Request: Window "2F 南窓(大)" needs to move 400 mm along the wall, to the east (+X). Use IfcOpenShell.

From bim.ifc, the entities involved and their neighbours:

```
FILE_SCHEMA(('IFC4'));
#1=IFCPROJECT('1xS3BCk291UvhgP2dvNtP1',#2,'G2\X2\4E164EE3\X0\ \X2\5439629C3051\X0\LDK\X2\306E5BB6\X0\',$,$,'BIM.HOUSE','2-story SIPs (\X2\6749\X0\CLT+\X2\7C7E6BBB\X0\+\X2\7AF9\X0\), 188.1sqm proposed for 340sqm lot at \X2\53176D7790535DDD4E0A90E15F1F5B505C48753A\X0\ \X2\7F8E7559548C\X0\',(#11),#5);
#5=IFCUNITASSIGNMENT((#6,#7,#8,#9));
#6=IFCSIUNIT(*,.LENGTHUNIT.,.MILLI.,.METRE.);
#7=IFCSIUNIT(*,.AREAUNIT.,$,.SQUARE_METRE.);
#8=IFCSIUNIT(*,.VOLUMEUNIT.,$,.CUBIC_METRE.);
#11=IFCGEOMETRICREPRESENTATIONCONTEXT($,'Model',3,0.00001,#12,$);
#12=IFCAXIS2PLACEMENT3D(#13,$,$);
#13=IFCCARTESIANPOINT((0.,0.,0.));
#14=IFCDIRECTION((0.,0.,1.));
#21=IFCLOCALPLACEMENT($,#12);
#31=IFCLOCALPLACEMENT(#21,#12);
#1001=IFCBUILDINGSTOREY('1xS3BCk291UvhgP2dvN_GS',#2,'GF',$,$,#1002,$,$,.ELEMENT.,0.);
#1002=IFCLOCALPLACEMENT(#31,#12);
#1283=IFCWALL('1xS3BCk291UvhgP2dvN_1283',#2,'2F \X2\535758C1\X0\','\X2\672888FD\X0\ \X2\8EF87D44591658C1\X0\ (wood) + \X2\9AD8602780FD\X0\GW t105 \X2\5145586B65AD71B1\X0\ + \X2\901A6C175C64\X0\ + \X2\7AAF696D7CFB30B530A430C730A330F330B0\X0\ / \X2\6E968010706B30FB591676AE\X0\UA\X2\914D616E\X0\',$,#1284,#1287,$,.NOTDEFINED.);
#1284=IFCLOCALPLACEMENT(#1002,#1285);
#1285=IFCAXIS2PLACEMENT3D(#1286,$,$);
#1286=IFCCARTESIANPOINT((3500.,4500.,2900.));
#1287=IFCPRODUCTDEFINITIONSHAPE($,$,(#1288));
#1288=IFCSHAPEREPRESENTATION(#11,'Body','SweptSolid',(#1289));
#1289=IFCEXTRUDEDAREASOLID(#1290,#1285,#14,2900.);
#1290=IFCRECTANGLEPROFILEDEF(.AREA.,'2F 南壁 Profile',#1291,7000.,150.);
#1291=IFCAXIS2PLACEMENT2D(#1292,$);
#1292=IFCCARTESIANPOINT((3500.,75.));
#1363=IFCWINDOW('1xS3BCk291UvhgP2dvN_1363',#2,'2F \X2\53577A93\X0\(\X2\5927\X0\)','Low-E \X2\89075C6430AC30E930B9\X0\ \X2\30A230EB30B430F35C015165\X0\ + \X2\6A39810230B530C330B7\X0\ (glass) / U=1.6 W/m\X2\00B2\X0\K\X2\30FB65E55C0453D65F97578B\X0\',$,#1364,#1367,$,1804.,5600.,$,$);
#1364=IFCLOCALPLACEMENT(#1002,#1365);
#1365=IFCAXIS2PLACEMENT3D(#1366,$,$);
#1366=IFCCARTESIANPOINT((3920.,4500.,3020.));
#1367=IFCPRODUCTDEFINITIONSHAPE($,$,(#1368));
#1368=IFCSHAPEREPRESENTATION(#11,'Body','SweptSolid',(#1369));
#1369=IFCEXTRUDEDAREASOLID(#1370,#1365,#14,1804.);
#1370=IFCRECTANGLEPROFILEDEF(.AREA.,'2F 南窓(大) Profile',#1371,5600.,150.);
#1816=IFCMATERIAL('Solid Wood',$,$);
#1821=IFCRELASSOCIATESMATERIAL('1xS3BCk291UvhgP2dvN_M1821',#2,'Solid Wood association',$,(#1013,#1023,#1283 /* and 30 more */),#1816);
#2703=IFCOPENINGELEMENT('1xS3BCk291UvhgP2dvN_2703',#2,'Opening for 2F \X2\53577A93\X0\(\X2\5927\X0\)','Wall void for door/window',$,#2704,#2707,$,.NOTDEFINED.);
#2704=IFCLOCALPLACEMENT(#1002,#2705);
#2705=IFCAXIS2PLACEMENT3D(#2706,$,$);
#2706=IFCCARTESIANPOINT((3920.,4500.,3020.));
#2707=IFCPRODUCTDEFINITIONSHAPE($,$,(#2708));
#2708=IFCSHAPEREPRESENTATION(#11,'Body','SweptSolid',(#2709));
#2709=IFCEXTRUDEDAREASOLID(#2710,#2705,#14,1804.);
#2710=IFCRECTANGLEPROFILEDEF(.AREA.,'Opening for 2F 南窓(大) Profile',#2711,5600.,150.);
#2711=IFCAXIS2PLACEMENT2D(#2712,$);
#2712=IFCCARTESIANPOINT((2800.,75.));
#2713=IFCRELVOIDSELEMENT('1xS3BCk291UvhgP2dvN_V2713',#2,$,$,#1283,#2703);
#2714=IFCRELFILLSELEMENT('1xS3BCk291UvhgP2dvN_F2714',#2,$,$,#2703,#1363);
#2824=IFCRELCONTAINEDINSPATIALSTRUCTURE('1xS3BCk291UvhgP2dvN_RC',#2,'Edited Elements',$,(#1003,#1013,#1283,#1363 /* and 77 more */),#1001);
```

```python
import ifcopenshell
import ifcopenshell.api.geometry
import ifcopenshell.util.placement

model = ifcopenshell.open("bim.ifc")

window = model.by_id(1363)
opening = window.FillsVoids[0].RelatingOpeningElement
wall = opening.VoidsElements[0].RelatingBuildingElement

wall_matrix = ifcopenshell.util.placement.get_local_placement(wall.ObjectPlacement)
shift = wall_matrix[:3, 0] * 400.0
before = ifcopenshell.util.placement.get_local_placement(window.ObjectPlacement)[:3, 3].copy()

# The window is not placed relative to its opening, so move both.
for product in (opening, window):
    matrix = ifcopenshell.util.placement.get_local_placement(product.ObjectPlacement)
    matrix[:3, 3] += shift
    ifcopenshell.api.geometry.edit_object_placement(model, product=product, matrix=matrix, is_si=False)

after = ifcopenshell.util.placement.get_local_placement(window.ObjectPlacement)[:3, 3]
print("window moved by", (after - before).round(3) + 0.0)

model.write("bim-out.ifc")
```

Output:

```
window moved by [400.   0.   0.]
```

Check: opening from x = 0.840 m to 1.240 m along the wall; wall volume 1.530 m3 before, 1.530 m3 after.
